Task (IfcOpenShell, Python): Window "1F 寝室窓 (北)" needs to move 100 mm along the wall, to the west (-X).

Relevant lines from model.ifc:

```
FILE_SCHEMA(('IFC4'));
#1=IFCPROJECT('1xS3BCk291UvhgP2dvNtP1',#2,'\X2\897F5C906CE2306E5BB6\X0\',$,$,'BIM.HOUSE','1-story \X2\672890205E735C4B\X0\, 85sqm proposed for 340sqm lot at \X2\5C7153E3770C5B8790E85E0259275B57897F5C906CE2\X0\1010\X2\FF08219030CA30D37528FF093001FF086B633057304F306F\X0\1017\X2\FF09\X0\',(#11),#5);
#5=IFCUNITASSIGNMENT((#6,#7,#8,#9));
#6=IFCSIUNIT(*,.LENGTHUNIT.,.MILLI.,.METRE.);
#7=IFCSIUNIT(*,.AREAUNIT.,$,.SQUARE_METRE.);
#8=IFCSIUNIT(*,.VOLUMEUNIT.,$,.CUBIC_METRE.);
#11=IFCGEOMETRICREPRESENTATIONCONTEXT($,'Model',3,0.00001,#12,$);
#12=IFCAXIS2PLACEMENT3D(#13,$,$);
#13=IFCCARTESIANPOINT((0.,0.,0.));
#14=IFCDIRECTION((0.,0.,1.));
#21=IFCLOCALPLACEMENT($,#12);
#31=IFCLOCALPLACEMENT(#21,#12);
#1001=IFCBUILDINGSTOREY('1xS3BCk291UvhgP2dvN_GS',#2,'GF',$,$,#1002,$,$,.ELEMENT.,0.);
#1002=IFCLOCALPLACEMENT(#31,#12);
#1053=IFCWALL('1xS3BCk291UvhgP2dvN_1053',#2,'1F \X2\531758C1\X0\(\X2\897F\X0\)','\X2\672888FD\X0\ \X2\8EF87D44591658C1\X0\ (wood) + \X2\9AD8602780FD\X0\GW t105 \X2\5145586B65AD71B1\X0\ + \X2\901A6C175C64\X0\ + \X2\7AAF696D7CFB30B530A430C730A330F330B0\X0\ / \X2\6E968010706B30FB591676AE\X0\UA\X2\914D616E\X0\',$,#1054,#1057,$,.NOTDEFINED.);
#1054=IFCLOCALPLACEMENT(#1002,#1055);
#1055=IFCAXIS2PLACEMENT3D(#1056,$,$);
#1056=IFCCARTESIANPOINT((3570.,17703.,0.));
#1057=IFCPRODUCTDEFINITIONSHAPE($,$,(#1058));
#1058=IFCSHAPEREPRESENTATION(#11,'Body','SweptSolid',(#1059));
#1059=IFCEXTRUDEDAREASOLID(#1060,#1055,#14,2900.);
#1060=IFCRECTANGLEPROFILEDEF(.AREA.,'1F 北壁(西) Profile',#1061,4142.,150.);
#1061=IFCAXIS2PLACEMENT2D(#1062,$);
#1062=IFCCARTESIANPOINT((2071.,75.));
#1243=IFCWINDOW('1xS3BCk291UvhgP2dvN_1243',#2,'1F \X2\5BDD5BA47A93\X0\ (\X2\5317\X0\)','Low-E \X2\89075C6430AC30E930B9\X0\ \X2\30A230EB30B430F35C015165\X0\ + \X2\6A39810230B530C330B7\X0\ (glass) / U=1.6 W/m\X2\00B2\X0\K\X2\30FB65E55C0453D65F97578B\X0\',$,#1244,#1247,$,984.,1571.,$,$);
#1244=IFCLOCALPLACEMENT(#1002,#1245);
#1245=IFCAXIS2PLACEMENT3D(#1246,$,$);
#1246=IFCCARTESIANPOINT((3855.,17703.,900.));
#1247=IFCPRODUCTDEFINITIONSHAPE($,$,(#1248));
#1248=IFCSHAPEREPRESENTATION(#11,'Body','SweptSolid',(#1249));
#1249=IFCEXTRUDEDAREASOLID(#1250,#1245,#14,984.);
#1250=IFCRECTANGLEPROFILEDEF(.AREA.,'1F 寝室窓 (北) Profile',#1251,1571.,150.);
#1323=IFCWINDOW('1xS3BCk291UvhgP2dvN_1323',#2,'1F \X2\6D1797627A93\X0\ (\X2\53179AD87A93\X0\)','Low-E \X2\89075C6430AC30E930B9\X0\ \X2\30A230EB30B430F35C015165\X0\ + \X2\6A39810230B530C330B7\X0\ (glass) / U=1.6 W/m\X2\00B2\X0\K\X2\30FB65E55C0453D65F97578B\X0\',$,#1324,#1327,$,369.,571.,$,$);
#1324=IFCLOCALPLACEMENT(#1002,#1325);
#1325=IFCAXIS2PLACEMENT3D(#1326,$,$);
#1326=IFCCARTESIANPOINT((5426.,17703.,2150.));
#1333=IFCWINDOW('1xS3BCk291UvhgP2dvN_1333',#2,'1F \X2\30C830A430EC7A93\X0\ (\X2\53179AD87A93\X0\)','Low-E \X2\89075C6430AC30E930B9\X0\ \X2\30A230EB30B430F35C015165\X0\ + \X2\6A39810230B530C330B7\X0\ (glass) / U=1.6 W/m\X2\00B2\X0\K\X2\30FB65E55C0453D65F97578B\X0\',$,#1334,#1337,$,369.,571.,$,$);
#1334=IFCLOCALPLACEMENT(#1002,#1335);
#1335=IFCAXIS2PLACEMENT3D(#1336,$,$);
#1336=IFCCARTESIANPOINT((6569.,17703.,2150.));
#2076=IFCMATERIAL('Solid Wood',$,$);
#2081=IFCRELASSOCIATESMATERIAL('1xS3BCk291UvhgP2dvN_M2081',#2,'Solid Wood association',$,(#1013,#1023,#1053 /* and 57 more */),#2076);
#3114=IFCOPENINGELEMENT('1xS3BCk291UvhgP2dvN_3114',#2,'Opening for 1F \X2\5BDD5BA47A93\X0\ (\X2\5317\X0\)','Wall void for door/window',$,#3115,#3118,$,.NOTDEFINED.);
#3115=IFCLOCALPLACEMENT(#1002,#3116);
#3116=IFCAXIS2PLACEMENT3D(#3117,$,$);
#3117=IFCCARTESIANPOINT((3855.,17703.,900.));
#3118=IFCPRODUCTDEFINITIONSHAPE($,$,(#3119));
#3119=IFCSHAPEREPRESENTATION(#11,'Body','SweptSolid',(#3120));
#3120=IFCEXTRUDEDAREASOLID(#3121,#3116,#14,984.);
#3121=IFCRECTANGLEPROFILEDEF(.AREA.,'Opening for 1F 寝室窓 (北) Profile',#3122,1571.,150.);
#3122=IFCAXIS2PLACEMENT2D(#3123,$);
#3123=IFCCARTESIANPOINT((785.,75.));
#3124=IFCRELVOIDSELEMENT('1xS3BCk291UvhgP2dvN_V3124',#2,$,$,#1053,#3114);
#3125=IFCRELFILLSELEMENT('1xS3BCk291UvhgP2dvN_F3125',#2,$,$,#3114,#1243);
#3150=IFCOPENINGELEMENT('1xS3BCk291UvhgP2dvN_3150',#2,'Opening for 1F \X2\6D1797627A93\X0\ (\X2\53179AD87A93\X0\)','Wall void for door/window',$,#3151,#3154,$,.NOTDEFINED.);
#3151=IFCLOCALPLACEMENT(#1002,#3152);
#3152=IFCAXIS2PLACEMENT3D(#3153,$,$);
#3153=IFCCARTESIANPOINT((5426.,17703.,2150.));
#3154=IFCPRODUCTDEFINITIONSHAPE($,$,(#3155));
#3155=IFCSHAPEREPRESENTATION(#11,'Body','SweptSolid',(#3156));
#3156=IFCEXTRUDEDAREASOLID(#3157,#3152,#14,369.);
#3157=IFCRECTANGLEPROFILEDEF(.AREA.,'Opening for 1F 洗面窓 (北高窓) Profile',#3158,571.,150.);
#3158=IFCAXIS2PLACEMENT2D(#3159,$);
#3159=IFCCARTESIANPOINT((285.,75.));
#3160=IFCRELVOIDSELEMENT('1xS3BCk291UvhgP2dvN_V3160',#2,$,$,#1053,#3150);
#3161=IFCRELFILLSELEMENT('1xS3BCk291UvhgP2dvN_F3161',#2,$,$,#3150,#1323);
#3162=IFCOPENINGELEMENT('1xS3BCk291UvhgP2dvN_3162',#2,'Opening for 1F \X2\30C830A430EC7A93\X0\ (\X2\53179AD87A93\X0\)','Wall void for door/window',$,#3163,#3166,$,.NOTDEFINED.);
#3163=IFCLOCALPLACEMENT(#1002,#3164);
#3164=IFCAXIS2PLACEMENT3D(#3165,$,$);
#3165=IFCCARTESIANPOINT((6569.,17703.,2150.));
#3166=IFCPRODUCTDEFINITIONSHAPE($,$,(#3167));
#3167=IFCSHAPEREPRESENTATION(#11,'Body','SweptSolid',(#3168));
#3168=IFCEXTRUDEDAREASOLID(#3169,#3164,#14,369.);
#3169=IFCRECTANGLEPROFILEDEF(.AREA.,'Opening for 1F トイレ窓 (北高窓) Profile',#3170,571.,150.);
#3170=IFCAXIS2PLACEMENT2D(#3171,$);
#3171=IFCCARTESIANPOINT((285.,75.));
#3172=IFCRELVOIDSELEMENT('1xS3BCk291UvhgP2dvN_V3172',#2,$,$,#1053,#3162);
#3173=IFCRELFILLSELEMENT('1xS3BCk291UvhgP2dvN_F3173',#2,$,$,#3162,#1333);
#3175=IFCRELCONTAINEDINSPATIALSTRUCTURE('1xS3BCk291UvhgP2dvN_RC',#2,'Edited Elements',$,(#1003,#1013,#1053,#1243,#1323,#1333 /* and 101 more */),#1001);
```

```python
import ifcopenshell
import ifcopenshell.api.geometry
import ifcopenshell.util.placement
import ifcopenshell.util.unit

model = ifcopenshell.open("model.ifc")
unit_scale = ifcopenshell.util.unit.calculate_unit_scale(model)

window = model.by_id(1243)
opening = window.FillsVoids[0].RelatingOpeningElement
wall = opening.VoidsElements[0].RelatingBuildingElement

wall_matrix = ifcopenshell.util.placement.get_local_placement(wall.ObjectPlacement)
shift = wall_matrix[:3, 0] * -0.1 / unit_scale
before = ifcopenshell.util.placement.get_local_placement(window.ObjectPlacement)[:3, 3].copy()

# The window is not placed relative to its opening, so move both.
for product in (opening, window):
    matrix = ifcopenshell.util.placement.get_local_placement(product.ObjectPlacement)
    matrix[:3, 3] += shift
    ifcopenshell.api.geometry.edit_object_placement(model, product=product, matrix=matrix, is_si=False)

after = ifcopenshell.util.placement.get_local_placement(window.ObjectPlacement)[:3, 3]
print("window moved by", (after - before).round(3) + 0.0)

model.write("model_v2.ifc")
```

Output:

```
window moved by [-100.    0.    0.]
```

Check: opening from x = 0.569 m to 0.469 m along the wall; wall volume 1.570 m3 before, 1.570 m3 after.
